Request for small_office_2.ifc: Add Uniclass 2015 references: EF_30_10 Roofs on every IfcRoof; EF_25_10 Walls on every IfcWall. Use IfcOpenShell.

First a look at what the model holds.

```python
import ifcopenshell

model = ifcopenshell.open("small_office_2.ifc")
print(model.schema)
print("classifications:", [c.Name for c in model.by_type("IfcClassification")])
for ifc_class in ("IfcDoor", "IfcRoof", "IfcStair", "IfcWall", "IfcWindow"):
    print(ifc_class, len(model.by_type(ifc_class)))
```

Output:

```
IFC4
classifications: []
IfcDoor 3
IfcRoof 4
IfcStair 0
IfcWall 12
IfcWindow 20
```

```python
import ifcopenshell
import ifcopenshell.api.classification

model = ifcopenshell.open("small_office_2.ifc")

system = ifcopenshell.api.classification.add_classification(model, classification="Uniclass 2015")

codes = {
    "IfcRoof": ("EF_30_10", "Roofs"),
    "IfcWall": ("EF_25_10", "Walls"),
}
for ifc_class, (code, name) in codes.items():
    products = model.by_type(ifc_class)
    ifcopenshell.api.classification.add_reference(
        model, products=products, classification=system, identification=code, name=name
    )
    print(code, len(products))

model.write("small_office_2_v2.ifc")
```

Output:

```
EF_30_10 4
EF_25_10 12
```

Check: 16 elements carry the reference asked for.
